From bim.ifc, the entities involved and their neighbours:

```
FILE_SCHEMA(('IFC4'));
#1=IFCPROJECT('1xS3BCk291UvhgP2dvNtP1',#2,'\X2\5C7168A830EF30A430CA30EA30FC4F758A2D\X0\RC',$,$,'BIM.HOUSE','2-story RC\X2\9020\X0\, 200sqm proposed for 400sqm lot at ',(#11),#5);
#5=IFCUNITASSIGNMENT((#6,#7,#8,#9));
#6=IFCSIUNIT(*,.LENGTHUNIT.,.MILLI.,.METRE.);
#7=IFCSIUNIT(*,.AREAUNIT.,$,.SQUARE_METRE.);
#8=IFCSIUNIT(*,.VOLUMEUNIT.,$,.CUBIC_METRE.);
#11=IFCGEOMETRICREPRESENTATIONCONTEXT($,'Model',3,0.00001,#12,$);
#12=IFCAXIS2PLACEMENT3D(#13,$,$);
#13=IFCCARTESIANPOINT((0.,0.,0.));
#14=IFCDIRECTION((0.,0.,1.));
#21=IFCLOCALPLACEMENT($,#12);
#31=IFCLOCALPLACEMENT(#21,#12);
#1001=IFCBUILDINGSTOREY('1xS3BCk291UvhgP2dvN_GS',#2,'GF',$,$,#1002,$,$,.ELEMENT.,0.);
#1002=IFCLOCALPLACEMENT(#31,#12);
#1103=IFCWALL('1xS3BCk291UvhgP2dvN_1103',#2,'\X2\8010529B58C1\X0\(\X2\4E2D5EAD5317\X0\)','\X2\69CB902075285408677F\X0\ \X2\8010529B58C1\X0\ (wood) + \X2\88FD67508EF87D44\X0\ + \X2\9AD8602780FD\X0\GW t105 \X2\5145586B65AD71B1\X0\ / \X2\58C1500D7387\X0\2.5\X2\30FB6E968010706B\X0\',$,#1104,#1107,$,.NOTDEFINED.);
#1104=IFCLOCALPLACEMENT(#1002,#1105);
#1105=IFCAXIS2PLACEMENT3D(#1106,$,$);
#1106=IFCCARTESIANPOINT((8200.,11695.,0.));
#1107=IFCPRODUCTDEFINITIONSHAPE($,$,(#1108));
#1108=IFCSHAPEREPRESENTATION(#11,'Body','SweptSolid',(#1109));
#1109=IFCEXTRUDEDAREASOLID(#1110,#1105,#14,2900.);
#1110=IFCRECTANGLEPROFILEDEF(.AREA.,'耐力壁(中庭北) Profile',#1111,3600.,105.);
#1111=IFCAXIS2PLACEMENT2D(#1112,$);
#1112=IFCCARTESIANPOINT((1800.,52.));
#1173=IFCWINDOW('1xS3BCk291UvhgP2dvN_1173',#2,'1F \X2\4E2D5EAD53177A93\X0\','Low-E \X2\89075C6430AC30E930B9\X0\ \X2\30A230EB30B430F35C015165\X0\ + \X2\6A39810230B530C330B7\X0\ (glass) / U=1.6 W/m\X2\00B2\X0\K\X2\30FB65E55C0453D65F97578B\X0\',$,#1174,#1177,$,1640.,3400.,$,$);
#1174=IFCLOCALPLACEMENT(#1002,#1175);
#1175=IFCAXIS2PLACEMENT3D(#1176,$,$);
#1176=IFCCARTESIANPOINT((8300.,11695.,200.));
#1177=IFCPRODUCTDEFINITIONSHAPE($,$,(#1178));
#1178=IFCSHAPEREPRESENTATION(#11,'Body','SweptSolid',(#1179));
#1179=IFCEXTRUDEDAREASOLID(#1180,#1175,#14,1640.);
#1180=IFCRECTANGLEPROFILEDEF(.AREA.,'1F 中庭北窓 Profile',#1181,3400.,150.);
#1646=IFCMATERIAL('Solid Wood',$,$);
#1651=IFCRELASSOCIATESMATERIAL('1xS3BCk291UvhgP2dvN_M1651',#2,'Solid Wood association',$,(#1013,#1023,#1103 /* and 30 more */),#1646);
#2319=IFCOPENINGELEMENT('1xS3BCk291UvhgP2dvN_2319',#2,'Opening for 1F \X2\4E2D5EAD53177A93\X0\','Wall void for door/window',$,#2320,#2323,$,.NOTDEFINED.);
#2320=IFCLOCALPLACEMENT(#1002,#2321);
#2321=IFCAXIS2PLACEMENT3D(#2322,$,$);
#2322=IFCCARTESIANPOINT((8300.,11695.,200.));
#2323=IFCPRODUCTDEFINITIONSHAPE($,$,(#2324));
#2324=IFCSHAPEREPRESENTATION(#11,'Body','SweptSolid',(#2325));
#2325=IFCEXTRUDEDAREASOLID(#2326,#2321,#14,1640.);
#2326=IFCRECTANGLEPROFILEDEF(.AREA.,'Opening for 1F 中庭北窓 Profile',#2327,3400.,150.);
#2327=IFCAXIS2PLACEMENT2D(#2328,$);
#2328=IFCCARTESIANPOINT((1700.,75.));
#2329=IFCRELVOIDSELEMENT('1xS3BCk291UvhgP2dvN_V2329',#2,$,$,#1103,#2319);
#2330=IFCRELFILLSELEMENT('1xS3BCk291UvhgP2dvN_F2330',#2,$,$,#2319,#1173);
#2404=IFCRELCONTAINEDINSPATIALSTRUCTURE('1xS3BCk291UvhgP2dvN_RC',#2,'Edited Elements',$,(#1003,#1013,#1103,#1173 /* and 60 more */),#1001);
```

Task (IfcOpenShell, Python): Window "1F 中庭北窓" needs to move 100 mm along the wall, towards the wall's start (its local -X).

```python
import ifcopenshell
import ifcopenshell.api.geometry
import ifcopenshell.util.placement
import ifcopenshell.util.unit

model = ifcopenshell.open("bim.ifc")
unit_scale = ifcopenshell.util.unit.calculate_unit_scale(model)

window = model.by_guid("1xS3BCk291UvhgP2dvN_1173")
opening = window.FillsVoids[0].RelatingOpeningElement
wall = opening.VoidsElements[0].RelatingBuildingElement

wall_matrix = ifcopenshell.util.placement.get_local_placement(wall.ObjectPlacement)
shift = wall_matrix[:3, 0] * -0.1 / unit_scale
before = ifcopenshell.util.placement.get_local_placement(window.ObjectPlacement)[:3, 3].copy()

# The window is not placed relative to its opening, so move both.
for product in (opening, window):
    matrix = ifcopenshell.util.placement.get_local_placement(product.ObjectPlacement)
    matrix[:3, 3] += shift
    ifcopenshell.api.geometry.edit_object_placement(model, product=product, matrix=matrix, is_si=False)

after = ifcopenshell.util.placement.get_local_placement(window.ObjectPlacement)[:3, 3]
print("window moved by", (after - before).round(3) + 0.0)

model.write("bim_edited.ifc")
```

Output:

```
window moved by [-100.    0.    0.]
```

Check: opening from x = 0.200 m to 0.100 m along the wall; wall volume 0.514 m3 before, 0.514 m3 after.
